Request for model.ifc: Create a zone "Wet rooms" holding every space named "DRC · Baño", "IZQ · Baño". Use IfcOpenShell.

First a look at what the model holds.

```python
import ifcopenshell

model = ifcopenshell.open("model.ifc")
print(model.schema)
seen = {}
for space in model.by_type("IfcSpace"):
    seen[space.LongName] = seen.get(space.LongName, 0) + 1
for name, count in sorted(seen.items(), key=str):
    print(count, "x", name)
print("zones:", [z.Name for z in model.by_type("IfcZone")][:20])
```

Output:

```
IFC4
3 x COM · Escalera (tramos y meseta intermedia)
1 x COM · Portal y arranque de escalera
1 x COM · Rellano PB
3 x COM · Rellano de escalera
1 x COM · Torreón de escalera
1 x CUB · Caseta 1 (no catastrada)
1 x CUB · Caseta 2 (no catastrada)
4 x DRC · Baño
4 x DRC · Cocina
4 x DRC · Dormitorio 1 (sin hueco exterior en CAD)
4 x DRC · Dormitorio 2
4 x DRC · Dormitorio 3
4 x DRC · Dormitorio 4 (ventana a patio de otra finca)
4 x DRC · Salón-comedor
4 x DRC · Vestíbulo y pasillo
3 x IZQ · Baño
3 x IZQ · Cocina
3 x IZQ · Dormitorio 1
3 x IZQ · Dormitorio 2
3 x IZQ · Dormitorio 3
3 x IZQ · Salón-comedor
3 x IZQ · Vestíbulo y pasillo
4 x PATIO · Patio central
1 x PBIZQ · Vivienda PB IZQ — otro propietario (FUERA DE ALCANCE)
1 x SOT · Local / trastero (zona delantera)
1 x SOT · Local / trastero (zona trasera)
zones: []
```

```python
import ifcopenshell
import ifcopenshell.api.group
import ifcopenshell.api.root

model = ifcopenshell.open("model.ifc")

names = {"DRC · Baño", "IZQ · Baño"}
spaces = [s for s in model.by_type("IfcSpace") if s.LongName in names]

zone = ifcopenshell.api.root.create_entity(model, ifc_class="IfcZone", name="Wet rooms")
ifcopenshell.api.group.assign_group(model, products=spaces, group=zone)
print(len(spaces), "spaces in", zone.Name)

model.write("model-out.ifc")
```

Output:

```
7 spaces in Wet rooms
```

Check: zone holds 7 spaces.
